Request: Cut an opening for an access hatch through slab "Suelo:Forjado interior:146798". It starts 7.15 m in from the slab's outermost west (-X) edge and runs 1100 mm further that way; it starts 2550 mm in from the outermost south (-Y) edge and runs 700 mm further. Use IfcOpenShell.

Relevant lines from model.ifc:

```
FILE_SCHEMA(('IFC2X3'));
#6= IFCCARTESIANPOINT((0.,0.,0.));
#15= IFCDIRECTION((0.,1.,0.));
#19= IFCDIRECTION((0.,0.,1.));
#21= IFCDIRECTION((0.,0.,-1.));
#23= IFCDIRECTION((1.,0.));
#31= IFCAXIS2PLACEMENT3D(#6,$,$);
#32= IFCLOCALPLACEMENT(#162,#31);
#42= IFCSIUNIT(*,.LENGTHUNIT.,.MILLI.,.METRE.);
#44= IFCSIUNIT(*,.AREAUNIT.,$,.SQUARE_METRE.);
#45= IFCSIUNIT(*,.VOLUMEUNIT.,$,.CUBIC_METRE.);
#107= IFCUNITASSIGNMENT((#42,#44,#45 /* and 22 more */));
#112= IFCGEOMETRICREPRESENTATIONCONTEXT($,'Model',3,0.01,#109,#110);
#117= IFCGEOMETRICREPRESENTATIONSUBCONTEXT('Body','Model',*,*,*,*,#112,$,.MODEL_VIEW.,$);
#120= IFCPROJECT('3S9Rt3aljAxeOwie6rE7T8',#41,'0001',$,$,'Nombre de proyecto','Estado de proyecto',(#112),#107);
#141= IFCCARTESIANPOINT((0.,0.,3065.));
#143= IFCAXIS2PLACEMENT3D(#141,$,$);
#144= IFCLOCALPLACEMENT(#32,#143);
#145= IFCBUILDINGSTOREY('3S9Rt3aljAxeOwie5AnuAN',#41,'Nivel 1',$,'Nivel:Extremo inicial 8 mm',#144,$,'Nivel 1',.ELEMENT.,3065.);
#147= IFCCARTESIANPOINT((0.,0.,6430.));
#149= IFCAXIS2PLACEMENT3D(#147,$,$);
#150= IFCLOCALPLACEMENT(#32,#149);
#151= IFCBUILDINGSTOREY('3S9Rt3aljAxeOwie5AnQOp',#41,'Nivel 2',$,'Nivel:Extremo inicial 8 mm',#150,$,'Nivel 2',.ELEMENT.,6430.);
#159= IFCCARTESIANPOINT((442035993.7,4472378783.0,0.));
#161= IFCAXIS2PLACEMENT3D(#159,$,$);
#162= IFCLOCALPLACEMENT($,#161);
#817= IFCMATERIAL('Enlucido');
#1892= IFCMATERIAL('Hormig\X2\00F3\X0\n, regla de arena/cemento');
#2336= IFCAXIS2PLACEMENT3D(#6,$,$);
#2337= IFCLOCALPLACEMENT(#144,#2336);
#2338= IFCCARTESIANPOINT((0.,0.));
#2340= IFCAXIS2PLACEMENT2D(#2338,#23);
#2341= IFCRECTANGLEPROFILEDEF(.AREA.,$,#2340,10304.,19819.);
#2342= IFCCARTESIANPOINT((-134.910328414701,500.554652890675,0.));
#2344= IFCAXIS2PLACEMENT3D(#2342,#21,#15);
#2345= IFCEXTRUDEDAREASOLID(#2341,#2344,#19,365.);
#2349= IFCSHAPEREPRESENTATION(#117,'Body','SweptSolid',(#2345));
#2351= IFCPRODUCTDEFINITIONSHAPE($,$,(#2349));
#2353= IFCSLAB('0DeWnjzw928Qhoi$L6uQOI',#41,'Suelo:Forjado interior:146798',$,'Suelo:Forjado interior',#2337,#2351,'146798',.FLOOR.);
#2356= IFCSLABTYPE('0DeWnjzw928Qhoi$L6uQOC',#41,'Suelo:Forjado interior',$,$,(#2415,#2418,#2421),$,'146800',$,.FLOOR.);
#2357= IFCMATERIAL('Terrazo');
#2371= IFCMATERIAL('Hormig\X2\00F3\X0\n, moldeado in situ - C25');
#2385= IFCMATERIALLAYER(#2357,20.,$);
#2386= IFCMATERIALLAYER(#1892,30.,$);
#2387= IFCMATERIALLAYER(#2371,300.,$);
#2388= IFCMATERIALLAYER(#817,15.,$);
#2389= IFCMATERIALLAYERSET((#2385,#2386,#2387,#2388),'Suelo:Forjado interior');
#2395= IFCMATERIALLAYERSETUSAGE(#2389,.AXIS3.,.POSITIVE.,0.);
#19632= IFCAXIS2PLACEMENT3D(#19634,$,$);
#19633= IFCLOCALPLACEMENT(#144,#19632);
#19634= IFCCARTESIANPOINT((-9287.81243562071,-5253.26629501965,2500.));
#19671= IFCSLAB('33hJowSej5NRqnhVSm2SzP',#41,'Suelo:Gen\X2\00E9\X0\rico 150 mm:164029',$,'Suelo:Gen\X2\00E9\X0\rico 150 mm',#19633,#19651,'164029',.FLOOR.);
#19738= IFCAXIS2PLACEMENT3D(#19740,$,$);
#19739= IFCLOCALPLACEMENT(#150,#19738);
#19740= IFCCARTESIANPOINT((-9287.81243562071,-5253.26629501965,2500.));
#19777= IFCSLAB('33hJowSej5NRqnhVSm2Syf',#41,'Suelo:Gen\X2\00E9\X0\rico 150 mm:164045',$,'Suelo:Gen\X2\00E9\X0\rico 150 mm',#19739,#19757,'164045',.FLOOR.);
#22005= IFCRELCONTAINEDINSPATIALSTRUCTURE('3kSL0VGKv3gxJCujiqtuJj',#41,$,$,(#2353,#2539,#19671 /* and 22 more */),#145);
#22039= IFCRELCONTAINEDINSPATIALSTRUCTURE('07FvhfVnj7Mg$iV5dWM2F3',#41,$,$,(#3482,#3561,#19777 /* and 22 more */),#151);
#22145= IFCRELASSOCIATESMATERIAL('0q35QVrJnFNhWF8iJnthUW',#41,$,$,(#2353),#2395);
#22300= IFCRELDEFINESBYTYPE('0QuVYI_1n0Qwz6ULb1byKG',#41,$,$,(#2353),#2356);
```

```python
import numpy as np
import ifcopenshell
import ifcopenshell.api.feature
import ifcopenshell.api.geometry
import ifcopenshell.api.root
import ifcopenshell.geom
import ifcopenshell.util.placement
import ifcopenshell.util.representation
import ifcopenshell.util.shape
import ifcopenshell.util.unit

model = ifcopenshell.open("model.ifc")
unit_scale = ifcopenshell.util.unit.calculate_unit_scale(model)
settings = ifcopenshell.geom.settings()


def volume(element):
    """Net volume in cubic metres, openings subtracted."""
    shape = ifcopenshell.geom.create_shape(settings, element)
    return ifcopenshell.util.shape.get_volume(shape.geometry)


slab = model.by_guid("0DeWnjzw928Qhoi$L6uQOI")
before = volume(slab)

# Extent in the slab's own axes, in metres. The edges named are its -X and -Y sides.
slab_shape = ifcopenshell.geom.create_shape(settings, slab)
vertices = ifcopenshell.util.shape.get_vertices(slab_shape.geometry)
x_min, y_min, bottom = vertices.min(axis=0)
top = vertices[:, 2].max()

opening = ifcopenshell.api.root.create_entity(model, ifc_class="IfcOpeningElement", name="Access hatch opening")
context = ifcopenshell.util.representation.get_context(model, "Model", "Body", "MODEL_VIEW")
width, depth = 1.1, 0.7
outline = [(0.0, 0.0), (width, 0.0), (width, depth), (0.0, depth), (0.0, 0.0)]
# Overshoot both faces by 50 mm so the cut is clean.
shape = ifcopenshell.api.geometry.add_slab_representation(
    model, context=context, depth=top - bottom + 0.1, polyline=outline
)
ifcopenshell.api.geometry.assign_representation(model, product=opening, representation=shape)

matrix = ifcopenshell.util.placement.get_local_placement(slab.ObjectPlacement)
matrix[:, 3] = matrix @ np.append(np.array([x_min + 7.15, y_min + 2.55, bottom - 0.05]) / unit_scale, 1.0)
ifcopenshell.api.geometry.edit_object_placement(model, product=opening, matrix=matrix, is_si=False)
ifcopenshell.api.feature.add_feature(model, feature=opening, element=slab)

after = volume(slab)

print(f"slab volume {before:.3f} -> {after:.3f} m3")

model.write("model_rev.ifc")
```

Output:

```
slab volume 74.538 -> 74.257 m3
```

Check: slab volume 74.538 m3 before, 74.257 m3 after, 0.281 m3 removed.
